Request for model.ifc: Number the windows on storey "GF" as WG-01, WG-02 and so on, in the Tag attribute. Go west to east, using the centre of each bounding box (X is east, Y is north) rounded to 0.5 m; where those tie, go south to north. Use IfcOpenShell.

First a look at what the model holds.

```python
import ifcopenshell
import ifcopenshell.util.element
import ifcopenshell.util.placement

model = ifcopenshell.open("model.ifc")
print(model.schema)
storey = next(s for s in model.by_type("IfcBuildingStorey") if s.Name == "GF")
windows = [e for e in ifcopenshell.util.element.get_decomposition(storey) if e.is_a("IfcWindow")]
for e in sorted(windows, key=lambda e: e.id()):
    origin = ifcopenshell.util.placement.get_local_placement(e.ObjectPlacement)[:3, 3]
    print(e.id(), e.Tag, e.Name, origin.round(2) + 0.0, sep=" | ")
```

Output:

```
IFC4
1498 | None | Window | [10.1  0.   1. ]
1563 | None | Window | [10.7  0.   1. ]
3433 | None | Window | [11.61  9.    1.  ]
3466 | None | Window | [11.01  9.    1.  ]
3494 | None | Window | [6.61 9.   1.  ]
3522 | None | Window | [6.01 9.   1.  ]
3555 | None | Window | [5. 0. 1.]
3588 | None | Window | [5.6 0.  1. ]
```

```python
import ifcopenshell
import ifcopenshell.geom
import ifcopenshell.util.element
import ifcopenshell.util.shape

model = ifcopenshell.open("model.ifc")
settings = ifcopenshell.geom.settings()
settings.set("use-world-coords", True)


def centre(element):
    shape = ifcopenshell.geom.create_shape(settings, element)
    return ifcopenshell.util.shape.get_bbox_centroid(shape.geometry)


storey = next(s for s in model.by_type("IfcBuildingStorey") if s.Name == "GF")
windows = [e for e in ifcopenshell.util.element.get_decomposition(storey) if e.is_a("IfcWindow")]

# Insertion points can sit at a corner or the storey origin, so sort by the geometry (in metres).
centres = {e: centre(e) for e in windows}
windows.sort(key=lambda e: (round(centres[e][0] / 0.5), centres[e][1]))

for i, e in enumerate(windows, start=1):
    number = f"WG-{i:02d}"
    e.Tag = number
    print(e.id(), number)

model.write("model_rev.ifc")
```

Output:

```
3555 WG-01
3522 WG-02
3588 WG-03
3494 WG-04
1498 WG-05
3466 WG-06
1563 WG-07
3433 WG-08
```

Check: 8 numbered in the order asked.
